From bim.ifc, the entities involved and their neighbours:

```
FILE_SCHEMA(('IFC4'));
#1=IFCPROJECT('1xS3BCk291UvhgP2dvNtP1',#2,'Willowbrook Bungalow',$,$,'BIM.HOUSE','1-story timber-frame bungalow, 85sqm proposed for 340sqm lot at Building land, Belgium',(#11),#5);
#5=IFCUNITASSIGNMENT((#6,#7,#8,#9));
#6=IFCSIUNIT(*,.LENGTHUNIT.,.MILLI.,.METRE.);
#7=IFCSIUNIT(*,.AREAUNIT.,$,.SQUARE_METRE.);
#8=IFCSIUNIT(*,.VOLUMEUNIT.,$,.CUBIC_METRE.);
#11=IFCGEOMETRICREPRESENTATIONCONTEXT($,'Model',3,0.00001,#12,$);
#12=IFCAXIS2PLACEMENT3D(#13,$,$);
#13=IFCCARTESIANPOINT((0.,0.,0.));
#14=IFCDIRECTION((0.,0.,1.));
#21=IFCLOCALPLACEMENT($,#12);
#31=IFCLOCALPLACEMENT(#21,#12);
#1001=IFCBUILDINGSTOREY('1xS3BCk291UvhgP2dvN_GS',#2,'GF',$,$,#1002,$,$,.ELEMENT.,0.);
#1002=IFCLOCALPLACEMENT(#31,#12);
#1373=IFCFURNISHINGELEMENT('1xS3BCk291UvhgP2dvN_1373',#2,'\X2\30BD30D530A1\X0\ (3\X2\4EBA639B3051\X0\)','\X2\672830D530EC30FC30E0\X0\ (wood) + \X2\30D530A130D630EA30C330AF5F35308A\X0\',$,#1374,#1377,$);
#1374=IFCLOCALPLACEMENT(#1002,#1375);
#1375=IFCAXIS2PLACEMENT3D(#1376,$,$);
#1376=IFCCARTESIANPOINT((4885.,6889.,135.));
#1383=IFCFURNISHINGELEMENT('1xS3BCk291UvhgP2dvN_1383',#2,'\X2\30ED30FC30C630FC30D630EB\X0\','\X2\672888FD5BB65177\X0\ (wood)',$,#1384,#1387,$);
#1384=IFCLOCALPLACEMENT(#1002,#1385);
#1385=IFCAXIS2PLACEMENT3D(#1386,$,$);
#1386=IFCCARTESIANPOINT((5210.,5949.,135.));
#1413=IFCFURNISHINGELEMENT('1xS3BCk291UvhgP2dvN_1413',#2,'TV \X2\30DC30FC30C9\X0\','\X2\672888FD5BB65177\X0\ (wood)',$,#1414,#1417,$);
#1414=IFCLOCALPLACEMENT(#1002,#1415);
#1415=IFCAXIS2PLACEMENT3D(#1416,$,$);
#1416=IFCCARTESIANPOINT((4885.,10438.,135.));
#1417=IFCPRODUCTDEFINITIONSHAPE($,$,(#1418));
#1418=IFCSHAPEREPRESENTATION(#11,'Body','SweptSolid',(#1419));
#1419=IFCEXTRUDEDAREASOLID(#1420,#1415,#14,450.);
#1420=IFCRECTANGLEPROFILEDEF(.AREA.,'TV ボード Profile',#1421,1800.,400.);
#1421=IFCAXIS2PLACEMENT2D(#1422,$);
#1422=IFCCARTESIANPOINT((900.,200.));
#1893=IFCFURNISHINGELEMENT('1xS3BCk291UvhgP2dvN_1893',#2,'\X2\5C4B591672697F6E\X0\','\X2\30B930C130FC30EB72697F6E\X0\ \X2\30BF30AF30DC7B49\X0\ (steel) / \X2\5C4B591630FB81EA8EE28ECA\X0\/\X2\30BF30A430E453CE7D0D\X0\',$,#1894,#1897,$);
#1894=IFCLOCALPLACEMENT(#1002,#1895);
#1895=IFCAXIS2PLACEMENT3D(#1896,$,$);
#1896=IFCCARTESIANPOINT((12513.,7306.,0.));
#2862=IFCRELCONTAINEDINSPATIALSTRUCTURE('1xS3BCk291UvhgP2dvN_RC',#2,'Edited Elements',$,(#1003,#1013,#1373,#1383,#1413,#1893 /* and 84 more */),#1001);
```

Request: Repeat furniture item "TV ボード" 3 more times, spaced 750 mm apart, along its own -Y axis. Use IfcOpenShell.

```python
import ifcopenshell
import ifcopenshell.api.geometry
import ifcopenshell.api.root
import ifcopenshell.util.element
import ifcopenshell.util.placement
import ifcopenshell.util.unit

model = ifcopenshell.open("bim.ifc")
unit_scale = ifcopenshell.util.unit.calculate_unit_scale(model)


def reuse_history(source, copy):
    """copy_class also copies each property set's owner history, people and application; keep the originals."""
    for rel in copy.IsDefinedBy:
        if rel.is_a("IfcRelDefinesByProperties") and (history := rel.RelatingPropertyDefinition.OwnerHistory):
            rel.RelatingPropertyDefinition.OwnerHistory = source.OwnerHistory
            ifcopenshell.util.element.remove_deep2(model, history)


source = model.by_guid("1xS3BCk291UvhgP2dvN_1413")
base = ifcopenshell.util.placement.get_local_placement(source.ObjectPlacement)
step = -base[:3, 1] * 0.75 / unit_scale

for i in range(1, 4):
    copy = ifcopenshell.api.root.copy_class(model, product=source)
    copy.Representation = ifcopenshell.util.element.copy_deep(
        model, source.Representation, exclude=["IfcGeometricRepresentationContext", "IfcRepresentationMap"]
    )
    reuse_history(source, copy)
    matrix = base.copy()
    matrix[:3, 3] += i * step
    print("added at", matrix[:3, 3].round(3) + 0.0)
    ifcopenshell.api.geometry.edit_object_placement(model, product=copy, matrix=matrix, is_si=False)

model.write("bim_edited.ifc")
```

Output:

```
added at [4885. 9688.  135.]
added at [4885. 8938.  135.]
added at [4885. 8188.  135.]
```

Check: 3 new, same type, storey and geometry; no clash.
